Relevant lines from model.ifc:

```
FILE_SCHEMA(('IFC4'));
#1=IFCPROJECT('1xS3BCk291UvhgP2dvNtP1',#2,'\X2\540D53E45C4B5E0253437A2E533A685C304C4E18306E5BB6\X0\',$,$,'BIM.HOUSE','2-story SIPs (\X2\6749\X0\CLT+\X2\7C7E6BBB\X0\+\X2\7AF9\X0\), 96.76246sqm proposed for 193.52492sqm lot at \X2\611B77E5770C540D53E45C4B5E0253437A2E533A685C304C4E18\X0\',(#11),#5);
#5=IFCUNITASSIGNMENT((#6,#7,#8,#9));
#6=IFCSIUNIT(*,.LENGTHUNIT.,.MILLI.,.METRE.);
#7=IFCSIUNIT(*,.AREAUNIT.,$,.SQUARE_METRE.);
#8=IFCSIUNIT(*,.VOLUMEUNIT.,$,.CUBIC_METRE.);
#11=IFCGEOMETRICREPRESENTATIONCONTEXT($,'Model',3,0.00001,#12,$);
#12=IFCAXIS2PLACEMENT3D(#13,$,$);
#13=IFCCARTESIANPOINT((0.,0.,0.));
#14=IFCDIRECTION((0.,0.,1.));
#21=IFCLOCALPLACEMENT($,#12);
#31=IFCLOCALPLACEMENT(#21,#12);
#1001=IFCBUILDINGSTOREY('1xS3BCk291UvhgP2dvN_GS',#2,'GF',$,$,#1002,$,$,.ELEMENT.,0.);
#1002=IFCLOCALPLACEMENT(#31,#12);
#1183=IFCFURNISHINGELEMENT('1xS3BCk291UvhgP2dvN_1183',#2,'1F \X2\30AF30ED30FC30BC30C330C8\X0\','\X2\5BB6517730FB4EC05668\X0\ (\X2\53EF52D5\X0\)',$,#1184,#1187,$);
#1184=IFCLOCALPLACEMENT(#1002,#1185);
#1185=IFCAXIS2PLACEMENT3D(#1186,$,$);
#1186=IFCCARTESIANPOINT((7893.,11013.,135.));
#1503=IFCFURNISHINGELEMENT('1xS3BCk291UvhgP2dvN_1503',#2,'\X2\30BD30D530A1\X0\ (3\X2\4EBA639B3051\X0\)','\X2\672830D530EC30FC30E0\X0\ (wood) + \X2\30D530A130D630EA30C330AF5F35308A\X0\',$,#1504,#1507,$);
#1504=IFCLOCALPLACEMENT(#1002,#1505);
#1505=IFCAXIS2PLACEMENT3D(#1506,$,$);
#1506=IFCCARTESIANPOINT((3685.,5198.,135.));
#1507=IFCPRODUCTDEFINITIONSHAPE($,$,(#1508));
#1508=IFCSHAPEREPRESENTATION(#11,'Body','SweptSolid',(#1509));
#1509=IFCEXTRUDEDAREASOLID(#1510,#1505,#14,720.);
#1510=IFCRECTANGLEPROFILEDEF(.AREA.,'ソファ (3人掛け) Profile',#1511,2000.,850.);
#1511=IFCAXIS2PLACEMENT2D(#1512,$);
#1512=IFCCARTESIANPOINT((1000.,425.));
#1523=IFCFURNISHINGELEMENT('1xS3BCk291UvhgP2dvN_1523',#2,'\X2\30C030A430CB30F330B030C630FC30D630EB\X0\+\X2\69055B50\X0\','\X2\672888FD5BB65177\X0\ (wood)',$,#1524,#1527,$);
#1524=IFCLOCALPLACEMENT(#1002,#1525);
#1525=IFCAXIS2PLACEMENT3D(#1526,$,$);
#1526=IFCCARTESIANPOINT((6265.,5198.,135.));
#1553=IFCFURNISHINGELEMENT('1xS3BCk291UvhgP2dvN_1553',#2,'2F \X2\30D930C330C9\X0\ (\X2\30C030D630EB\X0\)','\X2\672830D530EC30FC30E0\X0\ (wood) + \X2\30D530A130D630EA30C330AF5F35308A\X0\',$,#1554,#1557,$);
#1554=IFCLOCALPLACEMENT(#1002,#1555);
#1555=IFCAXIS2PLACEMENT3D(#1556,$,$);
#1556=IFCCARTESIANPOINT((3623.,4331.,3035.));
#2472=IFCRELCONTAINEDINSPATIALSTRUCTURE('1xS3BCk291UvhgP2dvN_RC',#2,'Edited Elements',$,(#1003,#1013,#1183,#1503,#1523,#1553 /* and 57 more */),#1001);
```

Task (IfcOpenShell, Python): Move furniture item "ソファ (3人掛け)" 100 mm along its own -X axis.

```python
import ifcopenshell
import ifcopenshell.api.geometry
import ifcopenshell.util.placement
import ifcopenshell.util.unit

model = ifcopenshell.open("model.ifc")
unit_scale = ifcopenshell.util.unit.calculate_unit_scale(model)

item = model.by_id(1503)
matrix = ifcopenshell.util.placement.get_local_placement(item.ObjectPlacement)
matrix[:3, 3] -= matrix[:3, 0] * 0.1 / unit_scale
ifcopenshell.api.geometry.edit_object_placement(model, product=item, matrix=matrix, is_si=False)

print(ifcopenshell.util.placement.get_local_placement(item.ObjectPlacement).round(3) + 0.0)

model.write("model_updated.ifc")
```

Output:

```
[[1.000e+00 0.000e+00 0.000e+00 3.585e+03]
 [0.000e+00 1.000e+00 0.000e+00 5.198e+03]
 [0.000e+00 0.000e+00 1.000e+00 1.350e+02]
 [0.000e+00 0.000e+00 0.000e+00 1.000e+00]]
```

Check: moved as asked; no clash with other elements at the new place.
